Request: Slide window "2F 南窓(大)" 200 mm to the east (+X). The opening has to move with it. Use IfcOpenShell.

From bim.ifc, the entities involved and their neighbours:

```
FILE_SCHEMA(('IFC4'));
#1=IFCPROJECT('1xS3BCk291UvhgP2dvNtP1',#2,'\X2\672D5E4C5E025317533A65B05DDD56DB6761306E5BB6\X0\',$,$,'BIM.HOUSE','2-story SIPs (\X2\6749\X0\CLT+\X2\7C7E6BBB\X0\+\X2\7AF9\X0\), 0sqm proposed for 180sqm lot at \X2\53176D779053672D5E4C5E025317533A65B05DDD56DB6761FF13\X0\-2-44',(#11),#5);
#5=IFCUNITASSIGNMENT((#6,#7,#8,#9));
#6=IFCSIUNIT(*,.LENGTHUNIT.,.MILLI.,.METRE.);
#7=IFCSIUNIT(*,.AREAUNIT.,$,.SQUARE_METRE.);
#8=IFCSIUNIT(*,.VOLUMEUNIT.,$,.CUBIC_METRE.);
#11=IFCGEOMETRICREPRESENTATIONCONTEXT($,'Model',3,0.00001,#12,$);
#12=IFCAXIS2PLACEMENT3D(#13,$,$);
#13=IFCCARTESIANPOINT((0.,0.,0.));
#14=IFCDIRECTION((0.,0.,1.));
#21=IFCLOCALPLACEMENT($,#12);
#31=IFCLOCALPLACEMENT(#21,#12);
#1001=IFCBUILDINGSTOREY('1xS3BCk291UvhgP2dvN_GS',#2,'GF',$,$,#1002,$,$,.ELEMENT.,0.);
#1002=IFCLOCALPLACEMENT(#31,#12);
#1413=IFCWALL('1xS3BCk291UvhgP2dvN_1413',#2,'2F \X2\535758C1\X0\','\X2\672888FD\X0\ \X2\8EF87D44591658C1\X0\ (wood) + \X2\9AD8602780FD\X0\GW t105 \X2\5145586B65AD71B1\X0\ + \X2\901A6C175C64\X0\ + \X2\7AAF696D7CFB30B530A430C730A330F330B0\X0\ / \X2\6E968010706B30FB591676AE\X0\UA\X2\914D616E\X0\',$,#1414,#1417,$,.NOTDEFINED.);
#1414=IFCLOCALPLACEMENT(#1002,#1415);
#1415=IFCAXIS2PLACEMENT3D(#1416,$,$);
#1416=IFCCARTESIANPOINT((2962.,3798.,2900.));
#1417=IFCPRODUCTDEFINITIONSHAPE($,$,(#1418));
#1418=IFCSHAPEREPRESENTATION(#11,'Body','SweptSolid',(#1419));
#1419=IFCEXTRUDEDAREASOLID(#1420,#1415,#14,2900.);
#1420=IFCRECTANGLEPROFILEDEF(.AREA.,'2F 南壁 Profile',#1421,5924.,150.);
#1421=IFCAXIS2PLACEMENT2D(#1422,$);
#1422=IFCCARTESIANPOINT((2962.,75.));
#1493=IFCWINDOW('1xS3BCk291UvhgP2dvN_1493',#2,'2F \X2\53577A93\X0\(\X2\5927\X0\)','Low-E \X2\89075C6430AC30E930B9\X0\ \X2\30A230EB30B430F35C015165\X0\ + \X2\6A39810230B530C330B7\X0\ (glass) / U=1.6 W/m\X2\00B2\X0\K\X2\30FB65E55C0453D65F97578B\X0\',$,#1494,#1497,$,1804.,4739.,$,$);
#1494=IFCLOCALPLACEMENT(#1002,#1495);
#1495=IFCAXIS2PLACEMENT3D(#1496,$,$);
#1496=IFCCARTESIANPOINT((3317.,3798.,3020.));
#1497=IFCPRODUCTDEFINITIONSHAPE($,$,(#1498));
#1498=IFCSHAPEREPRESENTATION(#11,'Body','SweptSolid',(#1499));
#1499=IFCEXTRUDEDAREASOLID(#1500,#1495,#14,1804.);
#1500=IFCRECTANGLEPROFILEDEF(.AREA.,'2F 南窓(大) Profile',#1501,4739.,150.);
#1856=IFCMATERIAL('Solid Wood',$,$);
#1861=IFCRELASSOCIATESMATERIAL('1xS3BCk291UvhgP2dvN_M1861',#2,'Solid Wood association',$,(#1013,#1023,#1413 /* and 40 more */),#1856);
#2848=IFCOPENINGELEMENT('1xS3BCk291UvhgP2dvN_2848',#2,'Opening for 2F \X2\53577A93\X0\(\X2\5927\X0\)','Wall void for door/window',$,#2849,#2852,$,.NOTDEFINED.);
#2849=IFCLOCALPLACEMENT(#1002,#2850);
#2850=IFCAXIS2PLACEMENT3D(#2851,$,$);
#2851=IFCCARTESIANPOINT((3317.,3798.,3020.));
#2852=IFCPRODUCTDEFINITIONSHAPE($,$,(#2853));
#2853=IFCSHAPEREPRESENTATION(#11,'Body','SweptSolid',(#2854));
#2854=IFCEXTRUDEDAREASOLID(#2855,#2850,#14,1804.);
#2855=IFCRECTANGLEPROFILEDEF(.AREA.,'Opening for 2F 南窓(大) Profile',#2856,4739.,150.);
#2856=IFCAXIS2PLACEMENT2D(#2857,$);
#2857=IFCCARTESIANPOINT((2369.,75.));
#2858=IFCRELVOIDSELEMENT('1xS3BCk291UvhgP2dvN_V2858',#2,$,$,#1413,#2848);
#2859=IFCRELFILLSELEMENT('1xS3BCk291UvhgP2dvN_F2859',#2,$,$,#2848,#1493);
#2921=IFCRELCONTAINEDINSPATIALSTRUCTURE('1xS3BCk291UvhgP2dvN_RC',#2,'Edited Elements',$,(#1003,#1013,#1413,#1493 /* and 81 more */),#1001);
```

```python
import ifcopenshell
import ifcopenshell.api.geometry
import ifcopenshell.util.placement
import ifcopenshell.util.unit

model = ifcopenshell.open("bim.ifc")
unit_scale = ifcopenshell.util.unit.calculate_unit_scale(model)

window = model.by_guid("1xS3BCk291UvhgP2dvN_1493")
opening = window.FillsVoids[0].RelatingOpeningElement
wall = opening.VoidsElements[0].RelatingBuildingElement

wall_matrix = ifcopenshell.util.placement.get_local_placement(wall.ObjectPlacement)
shift = wall_matrix[:3, 0] * 0.2 / unit_scale
before = ifcopenshell.util.placement.get_local_placement(window.ObjectPlacement)[:3, 3].copy()

# The window is not placed relative to its opening, so move both.
for product in (opening, window):
    matrix = ifcopenshell.util.placement.get_local_placement(product.ObjectPlacement)
    matrix[:3, 3] += shift
    ifcopenshell.api.geometry.edit_object_placement(model, product=product, matrix=matrix, is_si=False)

after = ifcopenshell.util.placement.get_local_placement(window.ObjectPlacement)[:3, 3]
print("window moved by", (after - before).round(3) + 0.0)

model.write("bim_updated.ifc")
```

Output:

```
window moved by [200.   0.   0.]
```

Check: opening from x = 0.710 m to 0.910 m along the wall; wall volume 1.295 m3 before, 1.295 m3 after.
